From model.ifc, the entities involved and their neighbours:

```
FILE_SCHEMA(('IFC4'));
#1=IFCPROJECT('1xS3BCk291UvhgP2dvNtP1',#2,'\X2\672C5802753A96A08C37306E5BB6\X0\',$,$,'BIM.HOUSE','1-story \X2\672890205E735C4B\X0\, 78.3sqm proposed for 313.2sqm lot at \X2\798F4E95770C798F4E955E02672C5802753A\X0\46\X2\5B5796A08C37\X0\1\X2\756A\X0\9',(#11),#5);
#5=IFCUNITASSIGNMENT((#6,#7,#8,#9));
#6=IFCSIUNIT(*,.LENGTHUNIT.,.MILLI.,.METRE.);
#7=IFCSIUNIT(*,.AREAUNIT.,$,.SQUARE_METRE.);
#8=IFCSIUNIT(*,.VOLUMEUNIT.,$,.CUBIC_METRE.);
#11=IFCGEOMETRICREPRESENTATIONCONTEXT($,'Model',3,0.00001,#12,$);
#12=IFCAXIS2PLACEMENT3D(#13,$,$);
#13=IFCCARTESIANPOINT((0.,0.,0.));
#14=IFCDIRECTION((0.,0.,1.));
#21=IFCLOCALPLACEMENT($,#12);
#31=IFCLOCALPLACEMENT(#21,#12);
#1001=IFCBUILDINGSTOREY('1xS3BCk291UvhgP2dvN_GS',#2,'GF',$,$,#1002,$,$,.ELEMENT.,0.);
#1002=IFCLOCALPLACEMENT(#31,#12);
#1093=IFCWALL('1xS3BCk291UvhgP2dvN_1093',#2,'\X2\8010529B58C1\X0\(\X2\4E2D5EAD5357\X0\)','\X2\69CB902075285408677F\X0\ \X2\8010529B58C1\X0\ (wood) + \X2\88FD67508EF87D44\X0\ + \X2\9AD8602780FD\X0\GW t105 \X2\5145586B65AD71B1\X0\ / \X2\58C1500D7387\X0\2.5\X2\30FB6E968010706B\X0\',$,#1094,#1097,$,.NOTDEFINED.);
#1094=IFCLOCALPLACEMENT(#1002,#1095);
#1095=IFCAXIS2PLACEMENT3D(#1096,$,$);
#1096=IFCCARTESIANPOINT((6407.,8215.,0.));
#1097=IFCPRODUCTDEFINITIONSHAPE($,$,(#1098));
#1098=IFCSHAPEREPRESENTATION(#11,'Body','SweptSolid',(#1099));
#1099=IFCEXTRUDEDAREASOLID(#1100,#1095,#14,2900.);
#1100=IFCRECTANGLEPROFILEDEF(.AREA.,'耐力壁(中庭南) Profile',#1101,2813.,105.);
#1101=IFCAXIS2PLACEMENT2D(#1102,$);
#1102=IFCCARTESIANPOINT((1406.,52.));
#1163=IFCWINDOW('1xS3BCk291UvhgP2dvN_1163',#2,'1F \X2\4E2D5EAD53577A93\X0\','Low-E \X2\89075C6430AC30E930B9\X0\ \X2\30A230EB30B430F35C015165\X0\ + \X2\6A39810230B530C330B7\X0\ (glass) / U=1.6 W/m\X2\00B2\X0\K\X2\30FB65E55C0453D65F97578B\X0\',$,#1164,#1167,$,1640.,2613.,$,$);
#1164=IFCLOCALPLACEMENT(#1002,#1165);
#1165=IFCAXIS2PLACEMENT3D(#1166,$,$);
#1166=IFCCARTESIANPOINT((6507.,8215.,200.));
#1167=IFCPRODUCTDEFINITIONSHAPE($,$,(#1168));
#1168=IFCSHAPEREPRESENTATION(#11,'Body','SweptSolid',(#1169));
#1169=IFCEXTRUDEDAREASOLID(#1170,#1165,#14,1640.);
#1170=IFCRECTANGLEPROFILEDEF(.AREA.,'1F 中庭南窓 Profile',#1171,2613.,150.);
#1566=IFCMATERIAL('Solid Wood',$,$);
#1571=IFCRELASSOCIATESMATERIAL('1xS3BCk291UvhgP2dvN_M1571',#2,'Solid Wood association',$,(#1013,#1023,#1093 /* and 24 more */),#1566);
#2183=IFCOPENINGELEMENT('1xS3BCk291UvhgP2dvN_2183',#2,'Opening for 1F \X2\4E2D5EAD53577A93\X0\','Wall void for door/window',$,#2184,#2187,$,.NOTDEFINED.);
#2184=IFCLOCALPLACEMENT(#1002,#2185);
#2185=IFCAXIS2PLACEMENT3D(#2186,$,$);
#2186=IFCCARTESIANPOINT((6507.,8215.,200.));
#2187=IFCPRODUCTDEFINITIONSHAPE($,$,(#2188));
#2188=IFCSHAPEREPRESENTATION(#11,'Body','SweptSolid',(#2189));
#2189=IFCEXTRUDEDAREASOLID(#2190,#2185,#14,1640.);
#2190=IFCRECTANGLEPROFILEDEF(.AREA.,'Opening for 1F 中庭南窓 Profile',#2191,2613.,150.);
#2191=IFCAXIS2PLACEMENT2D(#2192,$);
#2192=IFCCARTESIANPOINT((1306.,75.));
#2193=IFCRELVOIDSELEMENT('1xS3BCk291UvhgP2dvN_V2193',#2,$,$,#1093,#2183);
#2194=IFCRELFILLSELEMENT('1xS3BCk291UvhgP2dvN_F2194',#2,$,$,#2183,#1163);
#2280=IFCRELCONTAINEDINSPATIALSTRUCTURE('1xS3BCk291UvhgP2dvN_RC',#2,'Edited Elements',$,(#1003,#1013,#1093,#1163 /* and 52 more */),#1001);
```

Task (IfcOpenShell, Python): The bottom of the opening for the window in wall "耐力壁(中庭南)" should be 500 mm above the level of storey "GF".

```python
import numpy as np
import ifcopenshell
import ifcopenshell.api.geometry
import ifcopenshell.geom
import ifcopenshell.util.element
import ifcopenshell.util.placement
import ifcopenshell.util.shape
import ifcopenshell.util.unit

model = ifcopenshell.open("model.ifc")
unit_scale = ifcopenshell.util.unit.calculate_unit_scale(model)

window = model.by_guid("1xS3BCk291UvhgP2dvN_1163")
opening = window.FillsVoids[0].RelatingOpeningElement
storey = ifcopenshell.util.element.get_container(window, ifc_class="IfcBuildingStorey")
level = ifcopenshell.util.placement.get_local_placement(storey.ObjectPlacement)[2, 3]

# The opening's origin need not be at the sill, so measure its lowest point.
shape = ifcopenshell.geom.create_shape(ifcopenshell.geom.settings(), opening)
bottom = ifcopenshell.util.shape.get_shape_bottom_elevation(shape, shape.geometry) / unit_scale
dz = level + 500.0 - bottom

shift = np.array([0.0, 0.0, dz])
# The window is not placed relative to its opening, so move both.
for product in (opening, window):
    matrix = ifcopenshell.util.placement.get_local_placement(product.ObjectPlacement)
    matrix[:3, 3] += shift
    ifcopenshell.api.geometry.edit_object_placement(model, product=product, matrix=matrix, is_si=False)

print(f"moved by {dz * unit_scale:+.3f} m")

model.write("model_updated.ifc")
```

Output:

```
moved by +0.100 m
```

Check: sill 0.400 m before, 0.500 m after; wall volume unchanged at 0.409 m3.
